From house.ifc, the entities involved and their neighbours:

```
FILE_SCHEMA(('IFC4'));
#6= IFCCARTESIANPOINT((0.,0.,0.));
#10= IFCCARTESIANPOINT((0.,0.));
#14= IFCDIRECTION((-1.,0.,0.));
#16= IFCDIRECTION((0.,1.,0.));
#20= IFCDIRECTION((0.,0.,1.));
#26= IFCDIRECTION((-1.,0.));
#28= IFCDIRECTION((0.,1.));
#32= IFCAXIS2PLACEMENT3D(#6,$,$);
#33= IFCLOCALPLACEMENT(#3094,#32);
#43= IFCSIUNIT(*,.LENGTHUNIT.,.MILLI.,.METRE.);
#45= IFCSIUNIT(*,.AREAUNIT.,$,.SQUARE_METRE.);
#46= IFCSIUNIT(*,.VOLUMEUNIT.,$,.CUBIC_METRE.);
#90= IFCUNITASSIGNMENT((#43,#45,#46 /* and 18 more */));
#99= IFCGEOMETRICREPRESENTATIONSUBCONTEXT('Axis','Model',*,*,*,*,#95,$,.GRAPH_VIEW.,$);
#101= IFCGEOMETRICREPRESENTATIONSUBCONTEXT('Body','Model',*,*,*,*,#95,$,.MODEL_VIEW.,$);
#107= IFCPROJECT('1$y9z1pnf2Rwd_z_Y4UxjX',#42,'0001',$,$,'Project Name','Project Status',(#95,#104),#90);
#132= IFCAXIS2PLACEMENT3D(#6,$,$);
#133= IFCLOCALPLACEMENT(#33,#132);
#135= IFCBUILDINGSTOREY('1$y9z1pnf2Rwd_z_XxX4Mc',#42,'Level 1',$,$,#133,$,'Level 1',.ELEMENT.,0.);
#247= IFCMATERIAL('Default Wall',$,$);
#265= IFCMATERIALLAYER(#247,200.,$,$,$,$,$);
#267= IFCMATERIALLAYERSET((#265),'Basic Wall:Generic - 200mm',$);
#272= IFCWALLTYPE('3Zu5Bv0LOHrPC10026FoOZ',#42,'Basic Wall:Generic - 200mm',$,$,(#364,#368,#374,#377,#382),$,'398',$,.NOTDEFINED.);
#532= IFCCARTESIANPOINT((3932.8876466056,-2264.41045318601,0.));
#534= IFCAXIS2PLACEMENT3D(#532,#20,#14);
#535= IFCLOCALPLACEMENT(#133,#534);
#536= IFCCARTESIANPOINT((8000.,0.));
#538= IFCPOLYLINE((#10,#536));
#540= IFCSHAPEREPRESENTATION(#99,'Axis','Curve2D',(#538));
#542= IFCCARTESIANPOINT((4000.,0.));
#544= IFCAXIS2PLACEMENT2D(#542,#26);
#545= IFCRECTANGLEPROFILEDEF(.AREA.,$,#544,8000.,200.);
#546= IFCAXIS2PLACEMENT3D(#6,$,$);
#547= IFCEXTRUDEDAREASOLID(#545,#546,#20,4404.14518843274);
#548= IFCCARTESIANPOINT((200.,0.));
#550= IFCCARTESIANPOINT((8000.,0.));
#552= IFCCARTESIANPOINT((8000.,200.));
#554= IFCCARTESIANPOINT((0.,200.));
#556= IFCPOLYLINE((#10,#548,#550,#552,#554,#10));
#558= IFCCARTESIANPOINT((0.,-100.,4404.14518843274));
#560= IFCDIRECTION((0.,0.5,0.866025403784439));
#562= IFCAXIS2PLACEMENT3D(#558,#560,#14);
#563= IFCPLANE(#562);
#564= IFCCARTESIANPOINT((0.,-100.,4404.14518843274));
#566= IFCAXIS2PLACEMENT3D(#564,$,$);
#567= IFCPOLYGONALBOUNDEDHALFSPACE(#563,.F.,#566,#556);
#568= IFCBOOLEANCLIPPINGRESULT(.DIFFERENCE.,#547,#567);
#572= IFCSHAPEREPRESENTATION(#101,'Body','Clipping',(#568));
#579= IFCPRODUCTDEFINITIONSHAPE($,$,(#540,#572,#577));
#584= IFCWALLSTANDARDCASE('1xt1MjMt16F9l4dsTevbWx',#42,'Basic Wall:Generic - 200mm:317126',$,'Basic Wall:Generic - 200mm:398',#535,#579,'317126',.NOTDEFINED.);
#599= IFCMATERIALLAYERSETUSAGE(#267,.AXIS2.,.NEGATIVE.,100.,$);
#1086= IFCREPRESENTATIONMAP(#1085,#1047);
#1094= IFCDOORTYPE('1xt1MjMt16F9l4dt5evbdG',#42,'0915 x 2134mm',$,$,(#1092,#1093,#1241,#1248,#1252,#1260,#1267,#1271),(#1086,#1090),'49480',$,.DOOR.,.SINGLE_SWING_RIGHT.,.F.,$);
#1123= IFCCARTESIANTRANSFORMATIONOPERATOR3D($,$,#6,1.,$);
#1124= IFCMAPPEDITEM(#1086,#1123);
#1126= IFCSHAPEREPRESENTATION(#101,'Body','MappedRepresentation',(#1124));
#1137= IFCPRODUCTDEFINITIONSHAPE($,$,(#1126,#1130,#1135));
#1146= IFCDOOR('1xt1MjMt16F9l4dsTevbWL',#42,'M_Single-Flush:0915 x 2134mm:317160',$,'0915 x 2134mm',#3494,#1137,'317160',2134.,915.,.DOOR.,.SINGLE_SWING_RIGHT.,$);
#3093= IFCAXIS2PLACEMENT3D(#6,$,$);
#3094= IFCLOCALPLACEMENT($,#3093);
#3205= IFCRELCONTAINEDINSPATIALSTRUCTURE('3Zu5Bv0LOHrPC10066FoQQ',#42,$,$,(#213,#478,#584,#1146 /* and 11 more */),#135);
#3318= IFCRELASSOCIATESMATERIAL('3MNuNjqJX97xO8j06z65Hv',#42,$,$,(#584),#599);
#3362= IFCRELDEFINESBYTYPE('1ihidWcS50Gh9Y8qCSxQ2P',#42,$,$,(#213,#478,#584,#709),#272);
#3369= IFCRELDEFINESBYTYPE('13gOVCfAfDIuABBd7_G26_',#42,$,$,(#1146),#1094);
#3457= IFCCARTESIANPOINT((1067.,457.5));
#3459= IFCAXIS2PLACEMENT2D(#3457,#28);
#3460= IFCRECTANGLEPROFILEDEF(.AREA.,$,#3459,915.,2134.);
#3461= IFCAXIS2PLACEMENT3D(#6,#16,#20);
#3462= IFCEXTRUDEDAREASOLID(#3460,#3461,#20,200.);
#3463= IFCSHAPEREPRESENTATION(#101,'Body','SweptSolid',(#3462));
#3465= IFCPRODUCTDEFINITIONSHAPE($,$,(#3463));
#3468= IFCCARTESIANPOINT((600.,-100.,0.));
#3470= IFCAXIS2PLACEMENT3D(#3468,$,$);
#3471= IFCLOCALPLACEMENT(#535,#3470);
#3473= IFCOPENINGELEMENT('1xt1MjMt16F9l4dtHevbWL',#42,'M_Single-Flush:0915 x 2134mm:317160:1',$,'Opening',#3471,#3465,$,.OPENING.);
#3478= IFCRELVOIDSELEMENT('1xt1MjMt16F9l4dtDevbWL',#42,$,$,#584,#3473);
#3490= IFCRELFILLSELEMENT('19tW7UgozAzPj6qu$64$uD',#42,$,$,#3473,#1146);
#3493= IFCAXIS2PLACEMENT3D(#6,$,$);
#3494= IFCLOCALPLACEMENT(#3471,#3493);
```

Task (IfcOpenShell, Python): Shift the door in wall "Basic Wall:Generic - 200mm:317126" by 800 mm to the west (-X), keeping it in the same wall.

```python
import ifcopenshell
import ifcopenshell.api.geometry
import ifcopenshell.util.placement
import ifcopenshell.util.unit

model = ifcopenshell.open("house.ifc")
unit_scale = ifcopenshell.util.unit.calculate_unit_scale(model)

door = model.by_id(1146)
opening = door.FillsVoids[0].RelatingOpeningElement
wall = opening.VoidsElements[0].RelatingBuildingElement

wall_matrix = ifcopenshell.util.placement.get_local_placement(wall.ObjectPlacement)
shift = wall_matrix[:3, 0] * 0.8 / unit_scale
before = ifcopenshell.util.placement.get_local_placement(door.ObjectPlacement)[:3, 3].copy()

# The door is placed relative to its opening, so it follows when the opening moves.
matrix = ifcopenshell.util.placement.get_local_placement(opening.ObjectPlacement)
matrix[:3, 3] += shift
ifcopenshell.api.geometry.edit_object_placement(
    model, product=opening, matrix=matrix, is_si=False, should_transform_children=True
)

after = ifcopenshell.util.placement.get_local_placement(door.ObjectPlacement)[:3, 3]
print("door moved by", (after - before).round(3) + 0.0)

model.write("house_rev.ifc")
```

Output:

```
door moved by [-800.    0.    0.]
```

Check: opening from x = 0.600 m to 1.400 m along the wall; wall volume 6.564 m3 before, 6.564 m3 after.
